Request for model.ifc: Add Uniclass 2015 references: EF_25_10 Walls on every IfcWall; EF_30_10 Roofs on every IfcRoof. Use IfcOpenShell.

First a look at what the model holds.

```python
import ifcopenshell

model = ifcopenshell.open("model.ifc")
print(model.schema)
print("classifications:", [c.Name for c in model.by_type("IfcClassification")])
for ifc_class in ("IfcDoor", "IfcRoof", "IfcStair", "IfcWall", "IfcWindow"):
    print(ifc_class, len(model.by_type(ifc_class)))
```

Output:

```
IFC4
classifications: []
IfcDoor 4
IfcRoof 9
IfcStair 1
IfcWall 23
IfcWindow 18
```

```python
import ifcopenshell
import ifcopenshell.api.classification

model = ifcopenshell.open("model.ifc")

system = ifcopenshell.api.classification.add_classification(model, classification="Uniclass 2015")

codes = {
    "IfcWall": ("EF_25_10", "Walls"),
    "IfcRoof": ("EF_30_10", "Roofs"),
}
for ifc_class, (code, name) in codes.items():
    products = model.by_type(ifc_class)
    ifcopenshell.api.classification.add_reference(
        model, products=products, classification=system, identification=code, name=name
    )
    print(code, len(products))

model.write("model-out.ifc")
```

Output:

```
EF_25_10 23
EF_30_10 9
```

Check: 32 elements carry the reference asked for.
